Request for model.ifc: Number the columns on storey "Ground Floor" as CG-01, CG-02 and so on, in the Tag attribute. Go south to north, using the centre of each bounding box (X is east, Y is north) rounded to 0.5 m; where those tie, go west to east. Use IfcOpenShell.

First a look at what the model holds.

```python
import ifcopenshell
import ifcopenshell.util.element
import ifcopenshell.util.placement

model = ifcopenshell.open("model.ifc")
print(model.schema)
storey = next(s for s in model.by_type("IfcBuildingStorey") if s.Name == "Ground Floor")
columns = [e for e in ifcopenshell.util.element.get_decomposition(storey) if e.is_a("IfcColumn")]
for e in sorted(columns, key=lambda e: e.id()):
    origin = ifcopenshell.util.placement.get_local_placement(e.ObjectPlacement)[:3, 3]
    print(e.id(), e.Tag, e.Name, origin.round(2) + 0.0, sep=" | ")
```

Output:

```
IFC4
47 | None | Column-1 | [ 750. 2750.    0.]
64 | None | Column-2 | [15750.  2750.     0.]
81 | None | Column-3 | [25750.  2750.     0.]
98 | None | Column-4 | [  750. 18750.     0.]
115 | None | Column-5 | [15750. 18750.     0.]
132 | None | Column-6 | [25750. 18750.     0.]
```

```python
import ifcopenshell
import ifcopenshell.geom
import ifcopenshell.util.element
import ifcopenshell.util.shape

model = ifcopenshell.open("model.ifc")
settings = ifcopenshell.geom.settings()
settings.set("use-world-coords", True)


def centre(element):
    shape = ifcopenshell.geom.create_shape(settings, element)
    return ifcopenshell.util.shape.get_bbox_centroid(shape.geometry)


storey = next(s for s in model.by_type("IfcBuildingStorey") if s.Name == "Ground Floor")
columns = [e for e in ifcopenshell.util.element.get_decomposition(storey) if e.is_a("IfcColumn")]

# Insertion points can sit at a corner or the storey origin, so sort by the geometry (in metres).
centres = {e: centre(e) for e in columns}
columns.sort(key=lambda e: (round(centres[e][1] / 0.5), centres[e][0]))

for i, e in enumerate(columns, start=1):
    number = f"CG-{i:02d}"
    e.Tag = number
    print(e.id(), number)

model.write("model-out.ifc")
```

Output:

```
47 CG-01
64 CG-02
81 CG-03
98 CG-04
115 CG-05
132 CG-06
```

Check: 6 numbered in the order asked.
